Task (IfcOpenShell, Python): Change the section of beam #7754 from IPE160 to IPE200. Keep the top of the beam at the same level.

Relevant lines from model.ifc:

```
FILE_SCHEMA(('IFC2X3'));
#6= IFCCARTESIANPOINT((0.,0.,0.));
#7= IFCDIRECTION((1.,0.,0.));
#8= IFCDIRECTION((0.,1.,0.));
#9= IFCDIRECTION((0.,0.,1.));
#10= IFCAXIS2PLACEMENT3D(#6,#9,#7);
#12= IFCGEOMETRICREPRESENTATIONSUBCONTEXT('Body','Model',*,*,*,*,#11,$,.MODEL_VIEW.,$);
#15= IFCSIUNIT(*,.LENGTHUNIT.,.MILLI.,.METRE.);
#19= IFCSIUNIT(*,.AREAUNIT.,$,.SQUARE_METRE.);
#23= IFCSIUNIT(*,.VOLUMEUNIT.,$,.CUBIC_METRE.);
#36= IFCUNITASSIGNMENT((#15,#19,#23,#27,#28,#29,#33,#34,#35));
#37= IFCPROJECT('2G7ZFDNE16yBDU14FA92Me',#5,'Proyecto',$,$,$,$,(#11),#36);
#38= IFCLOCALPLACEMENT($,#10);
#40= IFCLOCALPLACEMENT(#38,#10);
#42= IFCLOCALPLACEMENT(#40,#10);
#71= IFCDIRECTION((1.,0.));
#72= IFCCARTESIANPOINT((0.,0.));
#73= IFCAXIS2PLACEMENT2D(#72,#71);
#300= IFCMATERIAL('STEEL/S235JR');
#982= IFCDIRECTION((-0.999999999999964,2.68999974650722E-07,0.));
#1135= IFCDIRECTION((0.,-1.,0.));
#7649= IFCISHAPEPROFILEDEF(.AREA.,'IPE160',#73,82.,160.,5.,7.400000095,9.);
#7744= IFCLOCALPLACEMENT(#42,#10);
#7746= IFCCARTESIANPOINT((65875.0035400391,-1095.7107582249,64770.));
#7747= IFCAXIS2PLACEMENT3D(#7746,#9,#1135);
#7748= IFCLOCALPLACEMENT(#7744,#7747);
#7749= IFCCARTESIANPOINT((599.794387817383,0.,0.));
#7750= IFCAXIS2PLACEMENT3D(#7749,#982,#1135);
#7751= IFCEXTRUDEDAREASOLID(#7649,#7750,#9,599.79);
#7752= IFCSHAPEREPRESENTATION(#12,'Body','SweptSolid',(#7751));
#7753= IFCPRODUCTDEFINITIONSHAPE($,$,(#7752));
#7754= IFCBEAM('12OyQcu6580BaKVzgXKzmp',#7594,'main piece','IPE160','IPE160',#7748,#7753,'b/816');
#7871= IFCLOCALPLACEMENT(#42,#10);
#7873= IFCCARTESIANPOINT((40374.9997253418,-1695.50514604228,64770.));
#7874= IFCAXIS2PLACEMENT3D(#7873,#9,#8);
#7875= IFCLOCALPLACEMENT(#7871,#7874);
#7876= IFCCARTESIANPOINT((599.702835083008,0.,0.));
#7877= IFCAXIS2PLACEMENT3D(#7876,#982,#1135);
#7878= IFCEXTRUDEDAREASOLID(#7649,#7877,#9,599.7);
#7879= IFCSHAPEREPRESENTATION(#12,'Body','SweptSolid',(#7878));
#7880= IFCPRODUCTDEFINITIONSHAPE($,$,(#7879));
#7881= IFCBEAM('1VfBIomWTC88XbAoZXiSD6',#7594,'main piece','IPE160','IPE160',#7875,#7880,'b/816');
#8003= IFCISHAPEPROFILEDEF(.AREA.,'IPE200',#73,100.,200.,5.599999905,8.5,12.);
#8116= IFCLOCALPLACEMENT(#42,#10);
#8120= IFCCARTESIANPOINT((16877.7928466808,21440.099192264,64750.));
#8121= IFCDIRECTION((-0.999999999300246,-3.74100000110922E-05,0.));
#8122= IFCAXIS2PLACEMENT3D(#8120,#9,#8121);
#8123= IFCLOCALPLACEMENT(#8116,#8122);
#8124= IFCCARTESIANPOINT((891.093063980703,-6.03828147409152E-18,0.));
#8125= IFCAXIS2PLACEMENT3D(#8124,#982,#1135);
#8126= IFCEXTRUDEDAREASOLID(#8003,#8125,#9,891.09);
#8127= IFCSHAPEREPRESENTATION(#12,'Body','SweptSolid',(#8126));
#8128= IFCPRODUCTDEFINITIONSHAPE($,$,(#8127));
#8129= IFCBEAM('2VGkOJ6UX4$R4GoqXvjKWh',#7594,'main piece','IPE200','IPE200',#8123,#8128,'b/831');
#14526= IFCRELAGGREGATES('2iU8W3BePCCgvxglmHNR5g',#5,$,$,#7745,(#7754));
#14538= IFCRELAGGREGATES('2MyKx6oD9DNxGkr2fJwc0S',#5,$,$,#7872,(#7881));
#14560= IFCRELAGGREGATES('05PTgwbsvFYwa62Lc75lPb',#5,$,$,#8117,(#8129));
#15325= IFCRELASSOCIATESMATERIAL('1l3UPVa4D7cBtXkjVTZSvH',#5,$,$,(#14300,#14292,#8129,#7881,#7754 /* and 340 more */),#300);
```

```python
import ifcopenshell
import ifcopenshell.util.element
import ifcopenshell.util.representation

model = ifcopenshell.open("model.ifc")

member = model.by_guid("12OyQcu6580BaKVzgXKzmp")
source = next(p for p in model.by_type("IfcIShapeProfileDef") if p.ProfileName == "IPE200")

body = ifcopenshell.util.representation.get_representation(member, "Model", "Body")
solid = body.Items[0]
old_profile = solid.SweptArea

# Copy the section's sizes but keep this member's own profile position.
profile = ifcopenshell.util.element.copy(model, source)
# Profiles are centred, so shift by half the change in depth to hold the top.
shift = (old_profile.OverallDepth - profile.OverallDepth) / 2
x, y = old_profile.Position.Location.Coordinates
up = (0.0, 1.0)  # upwards, in the solid's own plane
location = model.createIfcCartesianPoint((x + up[0] * shift, y + up[1] * shift))
profile.Position = model.createIfcAxis2Placement2D(location, old_profile.Position.RefDirection)
solid.SweptArea = profile
if not model.get_total_inverses(old_profile):
    ifcopenshell.util.element.remove_deep2(model, old_profile)
member.Description = member.Description.replace("IPE160", "IPE200")
member.ObjectType = member.ObjectType.replace("IPE160", "IPE200")

print(solid.SweptArea)

model.write("model-out.ifc")
```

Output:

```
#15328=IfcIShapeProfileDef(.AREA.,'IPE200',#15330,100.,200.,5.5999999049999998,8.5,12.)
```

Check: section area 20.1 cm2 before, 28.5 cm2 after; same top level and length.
